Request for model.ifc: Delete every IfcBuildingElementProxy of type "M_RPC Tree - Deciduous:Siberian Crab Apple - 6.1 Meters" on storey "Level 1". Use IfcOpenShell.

First a look at what the model holds.

```python
import ifcopenshell
import ifcopenshell.util.element

model = ifcopenshell.open("model.ifc")
print(model.schema)
storey = next(s for s in model.by_type("IfcBuildingStorey") if s.Name == "Level 1")
proxies = [e for e in ifcopenshell.util.element.get_decomposition(storey) if e.is_a("IfcBuildingElementProxy")]
seen = {}
for e in proxies:
    element_type = ifcopenshell.util.element.get_type(e)
    name = element_type.Name if element_type not in (None, e) else None
    seen[name] = seen.get(name, 0) + 1
for name, count in sorted(seen.items(), key=str):
    print(count, "x", name)
```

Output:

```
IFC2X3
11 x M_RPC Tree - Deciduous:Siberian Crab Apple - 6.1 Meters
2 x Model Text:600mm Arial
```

```python
import ifcopenshell
import ifcopenshell.api.root
import ifcopenshell.util.element

model = ifcopenshell.open("model.ifc")

storey = next(s for s in model.by_type("IfcBuildingStorey") if s.Name == "Level 1")
proxies = [e for e in ifcopenshell.util.element.get_decomposition(storey) if e.is_a("IfcBuildingElementProxy")]
targets = [e for e in proxies if (t := ifcopenshell.util.element.get_type(e)) not in (None, e) and t.Name == "M_RPC Tree - Deciduous:Siberian Crab Apple - 6.1 Meters"]

for e in targets:
    ifcopenshell.api.root.remove_product(model, product=e)
print(len(targets), "removed")

model.write("model_v2.ifc")
```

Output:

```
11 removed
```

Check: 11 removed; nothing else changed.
